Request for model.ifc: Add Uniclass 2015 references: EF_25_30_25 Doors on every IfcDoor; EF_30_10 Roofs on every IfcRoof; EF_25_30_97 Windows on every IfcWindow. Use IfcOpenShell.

First a look at what the model holds.

```python
import ifcopenshell

model = ifcopenshell.open("model.ifc")
print(model.schema)
print("classifications:", [c.Name for c in model.by_type("IfcClassification")])
for ifc_class in ("IfcDoor", "IfcRoof", "IfcStair", "IfcWall", "IfcWindow"):
    print(ifc_class, len(model.by_type(ifc_class)))
```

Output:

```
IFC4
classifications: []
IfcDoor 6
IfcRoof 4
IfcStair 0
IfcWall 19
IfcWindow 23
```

```python
import ifcopenshell
import ifcopenshell.api.classification

model = ifcopenshell.open("model.ifc")

system = ifcopenshell.api.classification.add_classification(model, classification="Uniclass 2015")

codes = {
    "IfcDoor": ("EF_25_30_25", "Doors"),
    "IfcRoof": ("EF_30_10", "Roofs"),
    "IfcWindow": ("EF_25_30_97", "Windows"),
}
for ifc_class, (code, name) in codes.items():
    products = model.by_type(ifc_class)
    ifcopenshell.api.classification.add_reference(
        model, products=products, classification=system, identification=code, name=name
    )
    print(code, len(products))

model.write("model_rev.ifc")
```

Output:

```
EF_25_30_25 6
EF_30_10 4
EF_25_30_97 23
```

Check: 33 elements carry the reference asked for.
